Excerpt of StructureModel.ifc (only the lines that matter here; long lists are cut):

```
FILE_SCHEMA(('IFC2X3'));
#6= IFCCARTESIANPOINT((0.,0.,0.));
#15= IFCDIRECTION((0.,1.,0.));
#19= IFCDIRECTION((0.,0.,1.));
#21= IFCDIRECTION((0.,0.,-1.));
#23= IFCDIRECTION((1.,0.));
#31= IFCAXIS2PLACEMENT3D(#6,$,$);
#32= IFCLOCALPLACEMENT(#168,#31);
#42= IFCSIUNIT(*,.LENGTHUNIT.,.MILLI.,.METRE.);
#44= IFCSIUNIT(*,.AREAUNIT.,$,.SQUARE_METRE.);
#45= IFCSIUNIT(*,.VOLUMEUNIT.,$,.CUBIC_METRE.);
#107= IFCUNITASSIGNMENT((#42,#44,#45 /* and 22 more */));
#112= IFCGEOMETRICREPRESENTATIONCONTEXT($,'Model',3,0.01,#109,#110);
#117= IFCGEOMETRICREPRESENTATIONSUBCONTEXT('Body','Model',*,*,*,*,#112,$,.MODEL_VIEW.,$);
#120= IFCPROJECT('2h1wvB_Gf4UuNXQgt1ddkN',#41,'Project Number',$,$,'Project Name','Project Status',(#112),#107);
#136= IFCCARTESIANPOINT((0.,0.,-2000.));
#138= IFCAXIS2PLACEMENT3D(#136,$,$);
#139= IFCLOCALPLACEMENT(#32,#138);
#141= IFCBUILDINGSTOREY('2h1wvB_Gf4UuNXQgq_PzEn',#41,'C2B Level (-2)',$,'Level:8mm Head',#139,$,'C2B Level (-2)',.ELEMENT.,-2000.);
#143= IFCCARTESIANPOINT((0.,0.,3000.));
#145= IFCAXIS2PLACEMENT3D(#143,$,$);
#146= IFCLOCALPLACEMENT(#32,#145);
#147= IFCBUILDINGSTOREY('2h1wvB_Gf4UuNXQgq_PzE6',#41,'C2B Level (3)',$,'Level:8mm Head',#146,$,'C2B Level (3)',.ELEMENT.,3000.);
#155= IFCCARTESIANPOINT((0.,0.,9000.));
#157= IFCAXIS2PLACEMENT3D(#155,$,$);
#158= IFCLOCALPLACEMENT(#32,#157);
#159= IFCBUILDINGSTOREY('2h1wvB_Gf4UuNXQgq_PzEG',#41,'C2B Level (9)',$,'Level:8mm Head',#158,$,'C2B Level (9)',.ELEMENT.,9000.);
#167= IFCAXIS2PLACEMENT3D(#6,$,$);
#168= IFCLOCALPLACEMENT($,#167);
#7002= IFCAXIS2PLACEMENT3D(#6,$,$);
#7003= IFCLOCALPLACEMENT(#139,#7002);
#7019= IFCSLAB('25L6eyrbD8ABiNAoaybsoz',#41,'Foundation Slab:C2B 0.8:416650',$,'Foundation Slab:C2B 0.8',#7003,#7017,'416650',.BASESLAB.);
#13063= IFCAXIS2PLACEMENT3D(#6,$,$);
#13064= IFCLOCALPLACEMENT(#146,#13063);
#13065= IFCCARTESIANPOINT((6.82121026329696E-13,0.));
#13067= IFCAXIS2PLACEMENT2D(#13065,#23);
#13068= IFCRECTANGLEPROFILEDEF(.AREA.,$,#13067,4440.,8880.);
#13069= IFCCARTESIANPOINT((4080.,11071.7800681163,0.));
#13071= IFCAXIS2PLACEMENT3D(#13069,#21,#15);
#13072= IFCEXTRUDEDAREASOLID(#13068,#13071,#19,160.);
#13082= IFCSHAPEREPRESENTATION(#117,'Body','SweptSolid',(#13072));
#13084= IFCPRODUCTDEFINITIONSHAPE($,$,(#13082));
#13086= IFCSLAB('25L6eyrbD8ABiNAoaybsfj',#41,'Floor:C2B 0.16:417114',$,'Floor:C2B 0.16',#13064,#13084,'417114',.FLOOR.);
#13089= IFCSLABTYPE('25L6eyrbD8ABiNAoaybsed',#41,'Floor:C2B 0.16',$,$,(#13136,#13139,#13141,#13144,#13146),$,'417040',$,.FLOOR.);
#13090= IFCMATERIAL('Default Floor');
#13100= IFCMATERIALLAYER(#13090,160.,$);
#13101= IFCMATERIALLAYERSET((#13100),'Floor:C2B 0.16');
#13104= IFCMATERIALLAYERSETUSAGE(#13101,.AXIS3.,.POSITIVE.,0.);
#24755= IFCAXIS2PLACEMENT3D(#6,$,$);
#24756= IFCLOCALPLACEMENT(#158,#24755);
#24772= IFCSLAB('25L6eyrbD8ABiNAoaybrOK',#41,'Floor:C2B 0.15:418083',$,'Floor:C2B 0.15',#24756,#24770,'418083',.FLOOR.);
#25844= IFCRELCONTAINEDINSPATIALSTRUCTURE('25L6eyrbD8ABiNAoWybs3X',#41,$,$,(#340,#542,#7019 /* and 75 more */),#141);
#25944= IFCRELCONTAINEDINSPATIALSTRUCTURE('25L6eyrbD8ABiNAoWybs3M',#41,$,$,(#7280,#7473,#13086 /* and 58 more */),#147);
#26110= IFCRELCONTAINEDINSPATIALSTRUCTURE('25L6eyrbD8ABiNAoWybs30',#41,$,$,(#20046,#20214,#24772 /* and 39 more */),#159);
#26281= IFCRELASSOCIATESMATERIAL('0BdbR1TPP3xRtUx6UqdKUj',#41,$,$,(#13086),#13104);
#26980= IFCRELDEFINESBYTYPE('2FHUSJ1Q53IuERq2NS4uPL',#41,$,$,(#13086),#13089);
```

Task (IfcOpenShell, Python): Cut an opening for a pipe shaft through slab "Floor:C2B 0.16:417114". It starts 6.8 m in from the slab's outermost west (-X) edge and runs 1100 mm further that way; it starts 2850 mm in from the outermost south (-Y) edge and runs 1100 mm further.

```python
import numpy as np
import ifcopenshell
import ifcopenshell.api.feature
import ifcopenshell.api.geometry
import ifcopenshell.api.root
import ifcopenshell.geom
import ifcopenshell.util.placement
import ifcopenshell.util.representation
import ifcopenshell.util.shape
import ifcopenshell.util.unit

model = ifcopenshell.open("StructureModel.ifc")
unit_scale = ifcopenshell.util.unit.calculate_unit_scale(model)
settings = ifcopenshell.geom.settings()


def volume(element):
    """Net volume in cubic metres, openings subtracted."""
    shape = ifcopenshell.geom.create_shape(settings, element)
    return ifcopenshell.util.shape.get_volume(shape.geometry)


slab = model.by_guid("25L6eyrbD8ABiNAoaybsfj")
before = volume(slab)

# Extent in the slab's own axes, in metres. The edges named are its -X and -Y sides.
slab_shape = ifcopenshell.geom.create_shape(settings, slab)
vertices = ifcopenshell.util.shape.get_vertices(slab_shape.geometry)
x_min, y_min, bottom = vertices.min(axis=0)
top = vertices[:, 2].max()

opening = ifcopenshell.api.root.create_entity(model, ifc_class="IfcOpeningElement", name="Pipe shaft opening")
context = ifcopenshell.util.representation.get_context(model, "Model", "Body", "MODEL_VIEW")
width, depth = 1.1, 1.1
outline = [(0.0, 0.0), (width, 0.0), (width, depth), (0.0, depth), (0.0, 0.0)]
# Overshoot both faces by 50 mm so the cut is clean.
shape = ifcopenshell.api.geometry.add_slab_representation(
    model, context=context, depth=top - bottom + 0.1, polyline=outline
)
ifcopenshell.api.geometry.assign_representation(model, product=opening, representation=shape)

matrix = ifcopenshell.util.placement.get_local_placement(slab.ObjectPlacement)
matrix[:, 3] = matrix @ np.append(np.array([x_min + 6.8, y_min + 2.85, bottom - 0.05]) / unit_scale, 1.0)
ifcopenshell.api.geometry.edit_object_placement(model, product=opening, matrix=matrix, is_si=False)
ifcopenshell.api.feature.add_feature(model, feature=opening, element=slab)

after = volume(slab)

print(f"slab volume {before:.3f} -> {after:.3f} m3")

model.write("StructureModel_edited.ifc")
```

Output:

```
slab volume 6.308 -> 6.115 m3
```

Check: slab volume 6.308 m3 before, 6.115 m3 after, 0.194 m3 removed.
